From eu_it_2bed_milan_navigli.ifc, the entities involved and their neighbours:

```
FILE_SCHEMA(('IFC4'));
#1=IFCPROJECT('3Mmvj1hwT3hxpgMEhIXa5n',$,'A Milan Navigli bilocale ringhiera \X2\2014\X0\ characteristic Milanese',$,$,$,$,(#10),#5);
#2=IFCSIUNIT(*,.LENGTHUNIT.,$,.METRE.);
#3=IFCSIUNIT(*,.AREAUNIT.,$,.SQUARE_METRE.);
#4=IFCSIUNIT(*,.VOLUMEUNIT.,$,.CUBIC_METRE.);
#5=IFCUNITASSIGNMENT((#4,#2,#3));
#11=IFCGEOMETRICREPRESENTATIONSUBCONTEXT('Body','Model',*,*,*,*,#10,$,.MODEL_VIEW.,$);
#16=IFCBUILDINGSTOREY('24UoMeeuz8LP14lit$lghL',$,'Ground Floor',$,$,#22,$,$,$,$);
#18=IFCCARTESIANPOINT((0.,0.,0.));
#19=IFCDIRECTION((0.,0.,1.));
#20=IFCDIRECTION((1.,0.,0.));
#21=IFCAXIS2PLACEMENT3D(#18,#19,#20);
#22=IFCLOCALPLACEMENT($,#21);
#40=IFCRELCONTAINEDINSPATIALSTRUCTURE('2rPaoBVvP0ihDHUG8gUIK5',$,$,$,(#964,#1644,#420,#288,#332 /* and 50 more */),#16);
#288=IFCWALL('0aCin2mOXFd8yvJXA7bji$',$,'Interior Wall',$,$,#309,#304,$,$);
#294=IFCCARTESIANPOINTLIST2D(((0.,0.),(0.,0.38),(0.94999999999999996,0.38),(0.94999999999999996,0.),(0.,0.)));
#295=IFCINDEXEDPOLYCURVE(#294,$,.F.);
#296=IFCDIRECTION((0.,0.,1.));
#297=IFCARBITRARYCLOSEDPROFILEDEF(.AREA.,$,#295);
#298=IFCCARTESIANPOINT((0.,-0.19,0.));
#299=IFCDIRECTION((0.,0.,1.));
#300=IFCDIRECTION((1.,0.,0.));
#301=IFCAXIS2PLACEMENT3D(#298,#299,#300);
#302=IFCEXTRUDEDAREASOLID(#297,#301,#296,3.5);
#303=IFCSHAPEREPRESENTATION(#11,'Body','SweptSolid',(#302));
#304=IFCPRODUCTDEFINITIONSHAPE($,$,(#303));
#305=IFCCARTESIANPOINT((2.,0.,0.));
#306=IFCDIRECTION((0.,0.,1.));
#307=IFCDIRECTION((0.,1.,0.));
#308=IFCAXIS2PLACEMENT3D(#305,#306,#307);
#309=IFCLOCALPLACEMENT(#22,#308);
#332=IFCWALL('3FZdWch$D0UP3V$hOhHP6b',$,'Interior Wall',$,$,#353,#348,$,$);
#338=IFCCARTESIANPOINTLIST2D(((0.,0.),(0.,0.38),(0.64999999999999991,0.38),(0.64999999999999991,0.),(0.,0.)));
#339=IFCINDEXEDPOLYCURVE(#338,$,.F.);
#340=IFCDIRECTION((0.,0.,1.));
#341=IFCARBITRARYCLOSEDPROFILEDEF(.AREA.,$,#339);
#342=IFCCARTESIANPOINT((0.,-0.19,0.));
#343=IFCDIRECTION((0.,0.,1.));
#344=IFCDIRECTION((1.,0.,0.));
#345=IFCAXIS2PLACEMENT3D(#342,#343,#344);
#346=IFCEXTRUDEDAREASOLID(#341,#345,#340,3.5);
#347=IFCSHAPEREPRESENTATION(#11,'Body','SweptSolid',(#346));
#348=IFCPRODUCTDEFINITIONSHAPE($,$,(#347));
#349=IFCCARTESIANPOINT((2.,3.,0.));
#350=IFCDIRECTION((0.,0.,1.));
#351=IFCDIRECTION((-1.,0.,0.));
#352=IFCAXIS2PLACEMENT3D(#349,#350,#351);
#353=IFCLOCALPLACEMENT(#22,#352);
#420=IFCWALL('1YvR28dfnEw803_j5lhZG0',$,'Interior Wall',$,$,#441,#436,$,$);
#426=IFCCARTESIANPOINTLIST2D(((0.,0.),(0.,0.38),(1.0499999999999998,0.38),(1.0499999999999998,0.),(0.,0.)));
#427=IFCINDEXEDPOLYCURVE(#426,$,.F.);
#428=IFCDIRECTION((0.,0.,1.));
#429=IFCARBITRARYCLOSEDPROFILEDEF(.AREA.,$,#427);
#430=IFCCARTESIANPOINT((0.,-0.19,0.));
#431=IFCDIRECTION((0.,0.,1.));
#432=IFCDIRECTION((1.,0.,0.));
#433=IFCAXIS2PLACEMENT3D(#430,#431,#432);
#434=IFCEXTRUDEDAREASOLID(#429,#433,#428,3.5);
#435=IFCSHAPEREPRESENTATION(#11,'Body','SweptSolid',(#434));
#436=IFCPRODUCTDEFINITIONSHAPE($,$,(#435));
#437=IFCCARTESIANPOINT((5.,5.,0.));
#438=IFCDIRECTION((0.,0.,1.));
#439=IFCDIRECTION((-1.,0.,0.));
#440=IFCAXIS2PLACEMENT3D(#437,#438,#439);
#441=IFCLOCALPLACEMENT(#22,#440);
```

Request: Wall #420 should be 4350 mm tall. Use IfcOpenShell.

```python
import ifcopenshell
import ifcopenshell.geom
import ifcopenshell.util.representation
import ifcopenshell.util.shape
import ifcopenshell.util.unit

model = ifcopenshell.open("eu_it_2bed_milan_navigli.ifc")
unit_scale = ifcopenshell.util.unit.calculate_unit_scale(model)
settings = ifcopenshell.geom.settings()


def volume(element):
    """Net volume in cubic metres, openings subtracted."""
    shape = ifcopenshell.geom.create_shape(settings, element)
    return ifcopenshell.util.shape.get_volume(shape.geometry)


wall = model.by_guid("1YvR28dfnEw803_j5lhZG0")
before = volume(wall)

body = ifcopenshell.util.representation.get_representation(wall, "Model", "Body")
solid = body.Items[0]
old_height = solid.Depth
solid.Depth = 4.35 / unit_scale
after = volume(wall)

print(f"height {old_height:g} -> {solid.Depth:g}, volume {before:.3f} -> {after:.3f} m3")

model.write("eu_it_2bed_milan_navigli-out.ifc")
```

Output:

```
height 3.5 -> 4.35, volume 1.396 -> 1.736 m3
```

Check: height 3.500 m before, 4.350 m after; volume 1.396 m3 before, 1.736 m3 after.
